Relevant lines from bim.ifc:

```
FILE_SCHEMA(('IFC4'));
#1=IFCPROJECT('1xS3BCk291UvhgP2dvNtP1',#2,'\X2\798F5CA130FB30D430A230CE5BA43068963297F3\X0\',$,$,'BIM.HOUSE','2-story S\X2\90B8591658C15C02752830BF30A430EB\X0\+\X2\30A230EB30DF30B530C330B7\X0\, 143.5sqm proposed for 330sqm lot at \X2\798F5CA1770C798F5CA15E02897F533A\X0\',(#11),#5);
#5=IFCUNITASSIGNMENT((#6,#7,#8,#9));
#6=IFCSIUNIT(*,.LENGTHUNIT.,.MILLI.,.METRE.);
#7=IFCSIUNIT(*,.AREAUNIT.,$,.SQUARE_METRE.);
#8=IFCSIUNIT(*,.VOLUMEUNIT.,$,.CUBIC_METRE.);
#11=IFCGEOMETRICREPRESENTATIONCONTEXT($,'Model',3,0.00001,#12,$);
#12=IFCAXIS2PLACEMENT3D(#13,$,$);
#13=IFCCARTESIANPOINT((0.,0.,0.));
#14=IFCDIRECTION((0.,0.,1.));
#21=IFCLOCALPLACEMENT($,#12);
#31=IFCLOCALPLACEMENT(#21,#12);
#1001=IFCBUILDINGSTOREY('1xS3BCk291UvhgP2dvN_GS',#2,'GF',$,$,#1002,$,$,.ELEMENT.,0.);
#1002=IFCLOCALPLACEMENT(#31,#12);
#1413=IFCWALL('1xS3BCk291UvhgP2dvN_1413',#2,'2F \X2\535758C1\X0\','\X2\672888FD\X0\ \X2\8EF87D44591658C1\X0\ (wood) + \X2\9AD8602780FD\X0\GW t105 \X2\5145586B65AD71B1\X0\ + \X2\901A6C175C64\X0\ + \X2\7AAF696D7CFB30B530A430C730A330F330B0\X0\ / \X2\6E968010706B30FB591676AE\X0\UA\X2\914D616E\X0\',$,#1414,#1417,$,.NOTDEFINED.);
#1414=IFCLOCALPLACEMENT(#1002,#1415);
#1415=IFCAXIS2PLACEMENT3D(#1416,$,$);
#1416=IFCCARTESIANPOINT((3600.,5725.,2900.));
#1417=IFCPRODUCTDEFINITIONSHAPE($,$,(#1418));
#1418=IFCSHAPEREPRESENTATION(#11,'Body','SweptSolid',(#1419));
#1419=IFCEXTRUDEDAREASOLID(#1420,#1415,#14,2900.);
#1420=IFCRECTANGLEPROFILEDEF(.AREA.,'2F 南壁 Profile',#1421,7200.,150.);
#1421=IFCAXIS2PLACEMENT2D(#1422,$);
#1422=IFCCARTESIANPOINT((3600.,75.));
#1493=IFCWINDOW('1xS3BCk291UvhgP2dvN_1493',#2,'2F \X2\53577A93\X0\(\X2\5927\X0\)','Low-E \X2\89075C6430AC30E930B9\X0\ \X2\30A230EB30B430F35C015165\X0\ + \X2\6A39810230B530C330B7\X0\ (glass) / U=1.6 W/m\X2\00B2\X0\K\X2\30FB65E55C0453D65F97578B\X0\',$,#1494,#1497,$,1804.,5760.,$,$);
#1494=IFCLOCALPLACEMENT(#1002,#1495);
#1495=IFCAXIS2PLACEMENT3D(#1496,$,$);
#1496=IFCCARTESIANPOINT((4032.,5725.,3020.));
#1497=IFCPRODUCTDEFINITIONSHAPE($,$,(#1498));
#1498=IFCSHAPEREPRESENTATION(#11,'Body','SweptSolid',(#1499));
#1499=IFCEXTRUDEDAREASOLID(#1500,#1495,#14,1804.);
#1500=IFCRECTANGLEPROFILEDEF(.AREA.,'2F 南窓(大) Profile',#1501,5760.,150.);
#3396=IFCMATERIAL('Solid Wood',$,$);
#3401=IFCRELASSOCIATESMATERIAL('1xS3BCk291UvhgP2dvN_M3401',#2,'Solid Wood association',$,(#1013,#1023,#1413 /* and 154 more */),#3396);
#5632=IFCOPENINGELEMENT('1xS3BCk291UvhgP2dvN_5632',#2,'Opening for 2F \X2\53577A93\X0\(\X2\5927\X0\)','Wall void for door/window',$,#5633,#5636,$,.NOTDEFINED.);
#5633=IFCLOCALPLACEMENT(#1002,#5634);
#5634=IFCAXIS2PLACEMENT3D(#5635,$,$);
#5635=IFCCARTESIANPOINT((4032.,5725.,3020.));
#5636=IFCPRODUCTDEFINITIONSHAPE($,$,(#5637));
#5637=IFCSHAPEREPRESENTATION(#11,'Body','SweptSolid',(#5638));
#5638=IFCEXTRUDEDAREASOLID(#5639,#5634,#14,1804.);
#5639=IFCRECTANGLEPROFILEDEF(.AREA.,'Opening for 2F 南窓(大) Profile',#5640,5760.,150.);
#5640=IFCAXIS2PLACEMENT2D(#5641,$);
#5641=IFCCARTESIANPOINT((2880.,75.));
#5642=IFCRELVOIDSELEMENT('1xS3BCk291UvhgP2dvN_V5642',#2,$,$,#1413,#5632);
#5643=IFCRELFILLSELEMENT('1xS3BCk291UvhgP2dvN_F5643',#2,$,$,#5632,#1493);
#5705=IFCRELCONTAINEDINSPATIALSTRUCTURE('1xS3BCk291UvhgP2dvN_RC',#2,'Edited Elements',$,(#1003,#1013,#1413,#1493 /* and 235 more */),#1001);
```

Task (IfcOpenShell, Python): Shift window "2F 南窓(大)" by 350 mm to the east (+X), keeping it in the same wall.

```python
import ifcopenshell
import ifcopenshell.api.geometry
import ifcopenshell.util.placement

model = ifcopenshell.open("bim.ifc")

window = model.by_id(1493)
opening = window.FillsVoids[0].RelatingOpeningElement
wall = opening.VoidsElements[0].RelatingBuildingElement

wall_matrix = ifcopenshell.util.placement.get_local_placement(wall.ObjectPlacement)
shift = wall_matrix[:3, 0] * 350.0
before = ifcopenshell.util.placement.get_local_placement(window.ObjectPlacement)[:3, 3].copy()

# The window is not placed relative to its opening, so move both.
for product in (opening, window):
    matrix = ifcopenshell.util.placement.get_local_placement(product.ObjectPlacement)
    matrix[:3, 3] += shift
    ifcopenshell.api.geometry.edit_object_placement(model, product=product, matrix=matrix, is_si=False)

after = ifcopenshell.util.placement.get_local_placement(window.ObjectPlacement)[:3, 3]
print("window moved by", (after - before).round(3) + 0.0)

model.write("bim_v2.ifc")
```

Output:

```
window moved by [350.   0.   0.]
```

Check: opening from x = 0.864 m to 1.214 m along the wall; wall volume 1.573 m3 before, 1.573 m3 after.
